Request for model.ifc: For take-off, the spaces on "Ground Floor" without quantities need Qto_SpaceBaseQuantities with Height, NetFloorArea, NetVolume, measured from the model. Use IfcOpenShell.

First a look at what the model holds.

```python
import ifcopenshell
import ifcopenshell.util.element
import ifcopenshell.util.unit

model = ifcopenshell.open("model.ifc")
print(model.schema)
for unit_type in ("LENGTHUNIT", "AREAUNIT", "VOLUMEUNIT"):
    print(unit_type, ifcopenshell.util.unit.calculate_unit_scale(model, unit_type))
storey = next(s for s in model.by_type("IfcBuildingStorey") if s.Name == "Ground Floor")
spaces = [e for e in ifcopenshell.util.element.get_decomposition(storey) if e.is_a("IfcSpace")]
for e in sorted(spaces, key=lambda e: e.id()):
    print(e.id(), e.is_a(), e.Name, list(ifcopenshell.util.element.get_psets(e, qtos_only=True)), sep=" | ")
```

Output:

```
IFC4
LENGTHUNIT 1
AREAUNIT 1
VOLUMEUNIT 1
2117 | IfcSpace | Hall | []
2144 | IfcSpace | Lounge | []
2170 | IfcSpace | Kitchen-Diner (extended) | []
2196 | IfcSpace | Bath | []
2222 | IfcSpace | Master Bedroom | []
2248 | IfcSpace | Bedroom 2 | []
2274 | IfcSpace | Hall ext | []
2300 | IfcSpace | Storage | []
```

```python
import ifcopenshell
import ifcopenshell.api.pset
import ifcopenshell.geom
import ifcopenshell.util.element
import ifcopenshell.util.shape
import ifcopenshell.util.unit

model = ifcopenshell.open("model.ifc")
unit_scale = ifcopenshell.util.unit.calculate_unit_scale(model)
area_scale = ifcopenshell.util.unit.calculate_unit_scale(model, "AREAUNIT")
volume_scale = ifcopenshell.util.unit.calculate_unit_scale(model, "VOLUMEUNIT")
settings = ifcopenshell.geom.settings()

storey = next(s for s in model.by_type("IfcBuildingStorey") if s.Name == "Ground Floor")
spaces = [e for e in ifcopenshell.util.element.get_decomposition(storey) if e.is_a("IfcSpace")]

for e in sorted(spaces, key=lambda e: e.id()):
    if ifcopenshell.util.element.get_psets(e, qtos_only=True, should_inherit=False):
        continue
    # Geometry comes back in metres, in the element's own axes.
    shape = ifcopenshell.geom.create_shape(settings, e)
    values = {
        "Height": ifcopenshell.util.shape.get_z(shape.geometry) / unit_scale,
        "NetFloorArea": ifcopenshell.util.shape.get_footprint_area(shape.geometry) / area_scale,
        "NetVolume": ifcopenshell.util.shape.get_volume(shape.geometry) / volume_scale,
    }
    qto = ifcopenshell.api.pset.add_qto(model, product=e, name="Qto_SpaceBaseQuantities")
    ifcopenshell.api.pset.edit_qto(model, qto=qto, properties=values)
    print(e.id(), {k: round(v, 3) for k, v in values.items()})

model.write("model_edited.ifc")
```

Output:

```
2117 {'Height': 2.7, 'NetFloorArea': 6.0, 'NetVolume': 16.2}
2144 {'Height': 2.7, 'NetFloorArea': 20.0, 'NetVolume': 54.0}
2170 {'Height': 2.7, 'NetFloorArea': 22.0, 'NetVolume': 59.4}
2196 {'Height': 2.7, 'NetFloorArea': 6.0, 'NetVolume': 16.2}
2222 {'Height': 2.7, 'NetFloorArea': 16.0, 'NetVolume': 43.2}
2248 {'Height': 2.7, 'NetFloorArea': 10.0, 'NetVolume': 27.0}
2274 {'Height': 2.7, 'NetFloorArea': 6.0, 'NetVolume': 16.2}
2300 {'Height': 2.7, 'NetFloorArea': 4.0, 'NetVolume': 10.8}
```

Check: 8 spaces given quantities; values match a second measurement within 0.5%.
